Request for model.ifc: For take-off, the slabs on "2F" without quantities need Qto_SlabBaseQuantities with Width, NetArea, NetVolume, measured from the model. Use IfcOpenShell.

First a look at what the model holds.

```python
import ifcopenshell
import ifcopenshell.util.element
import ifcopenshell.util.unit

model = ifcopenshell.open("model.ifc")
print(model.schema)
for unit_type in ("LENGTHUNIT", "AREAUNIT", "VOLUMEUNIT"):
    print(unit_type, ifcopenshell.util.unit.calculate_unit_scale(model, unit_type))
storey = next(s for s in model.by_type("IfcBuildingStorey") if s.Name == "2F")
slabs = [e for e in ifcopenshell.util.element.get_decomposition(storey) if e.is_a("IfcSlab")]
for e in sorted(slabs, key=lambda e: e.id()):
    print(e.id(), e.is_a(), e.Name, list(ifcopenshell.util.element.get_psets(e, qtos_only=True)), sep=" | ")
```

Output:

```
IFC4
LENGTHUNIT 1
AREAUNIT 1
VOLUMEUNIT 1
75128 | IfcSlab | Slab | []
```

```python
import ifcopenshell
import ifcopenshell.api.pset
import ifcopenshell.geom
import ifcopenshell.util.element
import ifcopenshell.util.shape
import ifcopenshell.util.unit

model = ifcopenshell.open("model.ifc")
unit_scale = ifcopenshell.util.unit.calculate_unit_scale(model)
area_scale = ifcopenshell.util.unit.calculate_unit_scale(model, "AREAUNIT")
volume_scale = ifcopenshell.util.unit.calculate_unit_scale(model, "VOLUMEUNIT")
settings = ifcopenshell.geom.settings()

storey = next(s for s in model.by_type("IfcBuildingStorey") if s.Name == "2F")
slabs = [e for e in ifcopenshell.util.element.get_decomposition(storey) if e.is_a("IfcSlab")]

for e in sorted(slabs, key=lambda e: e.id()):
    if ifcopenshell.util.element.get_psets(e, qtos_only=True, should_inherit=False):
        continue
    # Geometry comes back in metres, in the element's own axes.
    shape = ifcopenshell.geom.create_shape(settings, e)
    values = {
        "Width": ifcopenshell.util.shape.get_z(shape.geometry) / unit_scale,
        "NetArea": ifcopenshell.util.shape.get_footprint_area(shape.geometry) / area_scale,
        "NetVolume": ifcopenshell.util.shape.get_volume(shape.geometry) / volume_scale,
    }
    qto = ifcopenshell.api.pset.add_qto(model, product=e, name="Qto_SlabBaseQuantities")
    ifcopenshell.api.pset.edit_qto(model, qto=qto, properties=values)
    print(e.id(), {k: round(v, 3) for k, v in values.items()})

model.write("model-out.ifc")
```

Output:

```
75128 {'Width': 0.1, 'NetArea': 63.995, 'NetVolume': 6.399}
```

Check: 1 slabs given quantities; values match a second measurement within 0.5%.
